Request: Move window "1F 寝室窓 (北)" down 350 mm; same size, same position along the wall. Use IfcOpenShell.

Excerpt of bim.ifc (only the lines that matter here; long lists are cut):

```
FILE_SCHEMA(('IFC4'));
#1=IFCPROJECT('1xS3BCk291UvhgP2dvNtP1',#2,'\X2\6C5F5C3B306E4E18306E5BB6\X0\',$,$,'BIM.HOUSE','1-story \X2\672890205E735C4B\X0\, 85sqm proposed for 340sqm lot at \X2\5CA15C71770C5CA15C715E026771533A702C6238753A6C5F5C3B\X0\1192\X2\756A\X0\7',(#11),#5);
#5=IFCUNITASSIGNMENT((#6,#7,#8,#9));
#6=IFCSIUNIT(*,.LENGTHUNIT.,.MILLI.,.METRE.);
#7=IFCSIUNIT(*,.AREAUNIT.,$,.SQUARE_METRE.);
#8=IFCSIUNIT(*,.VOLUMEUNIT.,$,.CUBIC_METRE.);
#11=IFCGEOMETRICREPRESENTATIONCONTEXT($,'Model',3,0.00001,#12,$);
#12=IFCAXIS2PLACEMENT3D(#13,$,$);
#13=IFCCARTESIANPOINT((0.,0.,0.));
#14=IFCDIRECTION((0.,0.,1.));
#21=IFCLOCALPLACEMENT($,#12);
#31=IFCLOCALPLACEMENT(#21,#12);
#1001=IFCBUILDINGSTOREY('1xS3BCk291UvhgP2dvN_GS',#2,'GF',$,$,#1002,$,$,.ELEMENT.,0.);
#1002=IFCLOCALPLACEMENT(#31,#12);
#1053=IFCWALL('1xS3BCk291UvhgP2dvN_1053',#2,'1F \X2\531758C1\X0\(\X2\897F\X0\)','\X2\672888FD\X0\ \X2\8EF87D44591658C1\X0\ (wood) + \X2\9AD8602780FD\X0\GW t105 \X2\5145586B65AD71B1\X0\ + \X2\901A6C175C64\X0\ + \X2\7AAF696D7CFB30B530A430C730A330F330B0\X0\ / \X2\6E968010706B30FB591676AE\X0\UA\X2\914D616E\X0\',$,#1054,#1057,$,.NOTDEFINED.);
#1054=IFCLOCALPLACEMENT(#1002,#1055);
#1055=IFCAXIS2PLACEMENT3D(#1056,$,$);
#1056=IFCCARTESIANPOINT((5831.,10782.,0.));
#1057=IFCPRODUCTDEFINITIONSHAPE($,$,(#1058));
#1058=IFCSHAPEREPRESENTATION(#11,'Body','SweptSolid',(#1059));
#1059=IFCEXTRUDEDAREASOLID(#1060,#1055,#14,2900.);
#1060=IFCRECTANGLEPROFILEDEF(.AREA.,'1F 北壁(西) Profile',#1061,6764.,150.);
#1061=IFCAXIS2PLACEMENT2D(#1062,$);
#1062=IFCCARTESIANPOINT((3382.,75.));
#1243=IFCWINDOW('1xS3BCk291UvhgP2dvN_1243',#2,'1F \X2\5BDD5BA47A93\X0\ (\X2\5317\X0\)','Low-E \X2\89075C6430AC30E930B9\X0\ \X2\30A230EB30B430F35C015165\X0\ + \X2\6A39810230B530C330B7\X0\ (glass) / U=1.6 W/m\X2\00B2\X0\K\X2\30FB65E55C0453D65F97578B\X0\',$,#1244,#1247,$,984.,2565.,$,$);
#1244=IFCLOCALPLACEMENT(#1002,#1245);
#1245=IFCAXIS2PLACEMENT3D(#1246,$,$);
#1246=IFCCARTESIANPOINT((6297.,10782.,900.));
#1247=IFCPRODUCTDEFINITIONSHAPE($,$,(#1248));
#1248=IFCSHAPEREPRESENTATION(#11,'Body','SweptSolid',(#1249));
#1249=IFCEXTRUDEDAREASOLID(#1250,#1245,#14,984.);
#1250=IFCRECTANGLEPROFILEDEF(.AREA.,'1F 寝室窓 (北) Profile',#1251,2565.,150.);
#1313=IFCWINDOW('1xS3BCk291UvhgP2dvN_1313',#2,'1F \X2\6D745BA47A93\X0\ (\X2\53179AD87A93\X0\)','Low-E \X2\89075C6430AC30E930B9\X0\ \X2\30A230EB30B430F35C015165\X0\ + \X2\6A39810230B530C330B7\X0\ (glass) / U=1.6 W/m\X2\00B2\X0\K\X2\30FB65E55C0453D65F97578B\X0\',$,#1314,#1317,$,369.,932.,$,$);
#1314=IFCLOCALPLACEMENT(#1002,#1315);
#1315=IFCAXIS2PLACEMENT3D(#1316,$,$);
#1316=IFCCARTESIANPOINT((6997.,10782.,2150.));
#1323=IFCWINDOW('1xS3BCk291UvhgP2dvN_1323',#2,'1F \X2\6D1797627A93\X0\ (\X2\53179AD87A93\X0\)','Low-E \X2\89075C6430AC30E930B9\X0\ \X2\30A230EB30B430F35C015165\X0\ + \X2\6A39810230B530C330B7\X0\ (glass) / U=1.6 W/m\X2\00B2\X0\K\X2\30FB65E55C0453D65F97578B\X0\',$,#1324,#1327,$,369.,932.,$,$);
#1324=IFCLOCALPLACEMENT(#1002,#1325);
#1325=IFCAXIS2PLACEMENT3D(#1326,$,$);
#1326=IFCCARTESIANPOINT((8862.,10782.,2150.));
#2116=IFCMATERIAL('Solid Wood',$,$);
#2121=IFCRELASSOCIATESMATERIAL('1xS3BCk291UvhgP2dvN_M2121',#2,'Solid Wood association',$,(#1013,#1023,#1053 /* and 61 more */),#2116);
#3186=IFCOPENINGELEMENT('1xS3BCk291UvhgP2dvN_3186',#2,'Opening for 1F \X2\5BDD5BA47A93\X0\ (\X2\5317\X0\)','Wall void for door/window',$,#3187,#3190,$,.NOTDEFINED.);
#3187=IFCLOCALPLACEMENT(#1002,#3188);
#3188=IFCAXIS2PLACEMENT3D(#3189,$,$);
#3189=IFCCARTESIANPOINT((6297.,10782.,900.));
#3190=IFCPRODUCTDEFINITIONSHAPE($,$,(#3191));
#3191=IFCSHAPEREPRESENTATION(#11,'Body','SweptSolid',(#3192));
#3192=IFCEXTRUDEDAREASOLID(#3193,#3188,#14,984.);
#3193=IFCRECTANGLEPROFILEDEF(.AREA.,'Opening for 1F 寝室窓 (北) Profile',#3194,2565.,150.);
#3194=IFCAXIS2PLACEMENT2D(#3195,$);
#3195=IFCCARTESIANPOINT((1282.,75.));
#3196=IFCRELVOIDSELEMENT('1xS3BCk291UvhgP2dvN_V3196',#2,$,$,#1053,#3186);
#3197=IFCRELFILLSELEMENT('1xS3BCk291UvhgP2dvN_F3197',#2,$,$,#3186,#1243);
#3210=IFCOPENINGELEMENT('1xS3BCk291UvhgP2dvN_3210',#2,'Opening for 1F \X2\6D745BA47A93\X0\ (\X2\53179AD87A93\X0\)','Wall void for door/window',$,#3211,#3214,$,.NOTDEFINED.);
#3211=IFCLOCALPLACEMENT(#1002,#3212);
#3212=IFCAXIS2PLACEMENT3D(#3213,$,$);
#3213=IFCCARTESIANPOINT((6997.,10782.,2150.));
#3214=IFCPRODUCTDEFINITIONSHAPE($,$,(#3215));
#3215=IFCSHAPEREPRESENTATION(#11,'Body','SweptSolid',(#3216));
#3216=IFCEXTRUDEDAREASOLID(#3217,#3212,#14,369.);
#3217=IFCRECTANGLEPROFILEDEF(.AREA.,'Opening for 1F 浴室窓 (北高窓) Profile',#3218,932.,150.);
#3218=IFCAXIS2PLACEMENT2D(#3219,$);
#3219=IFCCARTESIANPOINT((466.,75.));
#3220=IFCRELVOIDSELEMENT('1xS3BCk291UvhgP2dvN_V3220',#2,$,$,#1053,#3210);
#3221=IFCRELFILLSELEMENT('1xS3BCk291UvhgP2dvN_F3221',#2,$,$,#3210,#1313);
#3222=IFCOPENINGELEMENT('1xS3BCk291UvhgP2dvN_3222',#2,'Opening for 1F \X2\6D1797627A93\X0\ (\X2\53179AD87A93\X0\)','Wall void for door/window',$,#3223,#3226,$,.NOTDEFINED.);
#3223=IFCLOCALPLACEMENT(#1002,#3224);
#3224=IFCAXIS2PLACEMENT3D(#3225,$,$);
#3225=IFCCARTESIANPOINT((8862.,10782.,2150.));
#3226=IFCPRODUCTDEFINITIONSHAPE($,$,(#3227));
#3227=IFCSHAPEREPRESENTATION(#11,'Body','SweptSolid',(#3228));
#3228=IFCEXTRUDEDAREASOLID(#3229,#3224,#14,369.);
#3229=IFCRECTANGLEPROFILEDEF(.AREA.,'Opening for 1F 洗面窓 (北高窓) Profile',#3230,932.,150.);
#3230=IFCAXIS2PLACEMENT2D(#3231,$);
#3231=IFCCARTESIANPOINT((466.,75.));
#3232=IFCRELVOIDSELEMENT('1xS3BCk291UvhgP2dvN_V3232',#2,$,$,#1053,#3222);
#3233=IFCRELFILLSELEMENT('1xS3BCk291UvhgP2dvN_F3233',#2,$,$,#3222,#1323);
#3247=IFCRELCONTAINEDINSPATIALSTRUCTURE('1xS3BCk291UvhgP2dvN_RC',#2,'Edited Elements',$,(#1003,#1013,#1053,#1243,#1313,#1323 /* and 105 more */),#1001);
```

```python
import numpy as np
import ifcopenshell
import ifcopenshell.api.geometry
import ifcopenshell.util.placement
import ifcopenshell.util.unit

model = ifcopenshell.open("bim.ifc")
unit_scale = ifcopenshell.util.unit.calculate_unit_scale(model)

window = model.by_guid("1xS3BCk291UvhgP2dvN_1243")
opening = window.FillsVoids[0].RelatingOpeningElement
dz = -0.35 / unit_scale

shift = np.array([0.0, 0.0, dz])
# The window is not placed relative to its opening, so move both.
for product in (opening, window):
    matrix = ifcopenshell.util.placement.get_local_placement(product.ObjectPlacement)
    matrix[:3, 3] += shift
    ifcopenshell.api.geometry.edit_object_placement(model, product=product, matrix=matrix, is_si=False)

print(f"moved by {dz * unit_scale:+.3f} m")

model.write("bim_v2.ifc")
```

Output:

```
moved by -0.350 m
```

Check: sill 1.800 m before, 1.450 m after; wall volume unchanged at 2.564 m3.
